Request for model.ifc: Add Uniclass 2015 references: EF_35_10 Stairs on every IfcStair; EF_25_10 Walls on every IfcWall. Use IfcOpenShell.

First a look at what the model holds.

```python
import ifcopenshell

model = ifcopenshell.open("model.ifc")
print(model.schema)
print("classifications:", [c.Name for c in model.by_type("IfcClassification")])
for ifc_class in ("IfcDoor", "IfcRoof", "IfcStair", "IfcWall", "IfcWindow"):
    print(ifc_class, len(model.by_type(ifc_class)))
```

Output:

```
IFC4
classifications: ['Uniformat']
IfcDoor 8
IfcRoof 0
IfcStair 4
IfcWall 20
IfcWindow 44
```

```python
import ifcopenshell
import ifcopenshell.api.classification

model = ifcopenshell.open("model.ifc")

system = ifcopenshell.api.classification.add_classification(model, classification="Uniclass 2015")

codes = {
    "IfcStair": ("EF_35_10", "Stairs"),
    "IfcWall": ("EF_25_10", "Walls"),
}
for ifc_class, (code, name) in codes.items():
    products = model.by_type(ifc_class)
    ifcopenshell.api.classification.add_reference(
        model, products=products, classification=system, identification=code, name=name
    )
    print(code, len(products))

model.write("model_edited.ifc")
```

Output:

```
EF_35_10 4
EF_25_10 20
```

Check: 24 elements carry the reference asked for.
